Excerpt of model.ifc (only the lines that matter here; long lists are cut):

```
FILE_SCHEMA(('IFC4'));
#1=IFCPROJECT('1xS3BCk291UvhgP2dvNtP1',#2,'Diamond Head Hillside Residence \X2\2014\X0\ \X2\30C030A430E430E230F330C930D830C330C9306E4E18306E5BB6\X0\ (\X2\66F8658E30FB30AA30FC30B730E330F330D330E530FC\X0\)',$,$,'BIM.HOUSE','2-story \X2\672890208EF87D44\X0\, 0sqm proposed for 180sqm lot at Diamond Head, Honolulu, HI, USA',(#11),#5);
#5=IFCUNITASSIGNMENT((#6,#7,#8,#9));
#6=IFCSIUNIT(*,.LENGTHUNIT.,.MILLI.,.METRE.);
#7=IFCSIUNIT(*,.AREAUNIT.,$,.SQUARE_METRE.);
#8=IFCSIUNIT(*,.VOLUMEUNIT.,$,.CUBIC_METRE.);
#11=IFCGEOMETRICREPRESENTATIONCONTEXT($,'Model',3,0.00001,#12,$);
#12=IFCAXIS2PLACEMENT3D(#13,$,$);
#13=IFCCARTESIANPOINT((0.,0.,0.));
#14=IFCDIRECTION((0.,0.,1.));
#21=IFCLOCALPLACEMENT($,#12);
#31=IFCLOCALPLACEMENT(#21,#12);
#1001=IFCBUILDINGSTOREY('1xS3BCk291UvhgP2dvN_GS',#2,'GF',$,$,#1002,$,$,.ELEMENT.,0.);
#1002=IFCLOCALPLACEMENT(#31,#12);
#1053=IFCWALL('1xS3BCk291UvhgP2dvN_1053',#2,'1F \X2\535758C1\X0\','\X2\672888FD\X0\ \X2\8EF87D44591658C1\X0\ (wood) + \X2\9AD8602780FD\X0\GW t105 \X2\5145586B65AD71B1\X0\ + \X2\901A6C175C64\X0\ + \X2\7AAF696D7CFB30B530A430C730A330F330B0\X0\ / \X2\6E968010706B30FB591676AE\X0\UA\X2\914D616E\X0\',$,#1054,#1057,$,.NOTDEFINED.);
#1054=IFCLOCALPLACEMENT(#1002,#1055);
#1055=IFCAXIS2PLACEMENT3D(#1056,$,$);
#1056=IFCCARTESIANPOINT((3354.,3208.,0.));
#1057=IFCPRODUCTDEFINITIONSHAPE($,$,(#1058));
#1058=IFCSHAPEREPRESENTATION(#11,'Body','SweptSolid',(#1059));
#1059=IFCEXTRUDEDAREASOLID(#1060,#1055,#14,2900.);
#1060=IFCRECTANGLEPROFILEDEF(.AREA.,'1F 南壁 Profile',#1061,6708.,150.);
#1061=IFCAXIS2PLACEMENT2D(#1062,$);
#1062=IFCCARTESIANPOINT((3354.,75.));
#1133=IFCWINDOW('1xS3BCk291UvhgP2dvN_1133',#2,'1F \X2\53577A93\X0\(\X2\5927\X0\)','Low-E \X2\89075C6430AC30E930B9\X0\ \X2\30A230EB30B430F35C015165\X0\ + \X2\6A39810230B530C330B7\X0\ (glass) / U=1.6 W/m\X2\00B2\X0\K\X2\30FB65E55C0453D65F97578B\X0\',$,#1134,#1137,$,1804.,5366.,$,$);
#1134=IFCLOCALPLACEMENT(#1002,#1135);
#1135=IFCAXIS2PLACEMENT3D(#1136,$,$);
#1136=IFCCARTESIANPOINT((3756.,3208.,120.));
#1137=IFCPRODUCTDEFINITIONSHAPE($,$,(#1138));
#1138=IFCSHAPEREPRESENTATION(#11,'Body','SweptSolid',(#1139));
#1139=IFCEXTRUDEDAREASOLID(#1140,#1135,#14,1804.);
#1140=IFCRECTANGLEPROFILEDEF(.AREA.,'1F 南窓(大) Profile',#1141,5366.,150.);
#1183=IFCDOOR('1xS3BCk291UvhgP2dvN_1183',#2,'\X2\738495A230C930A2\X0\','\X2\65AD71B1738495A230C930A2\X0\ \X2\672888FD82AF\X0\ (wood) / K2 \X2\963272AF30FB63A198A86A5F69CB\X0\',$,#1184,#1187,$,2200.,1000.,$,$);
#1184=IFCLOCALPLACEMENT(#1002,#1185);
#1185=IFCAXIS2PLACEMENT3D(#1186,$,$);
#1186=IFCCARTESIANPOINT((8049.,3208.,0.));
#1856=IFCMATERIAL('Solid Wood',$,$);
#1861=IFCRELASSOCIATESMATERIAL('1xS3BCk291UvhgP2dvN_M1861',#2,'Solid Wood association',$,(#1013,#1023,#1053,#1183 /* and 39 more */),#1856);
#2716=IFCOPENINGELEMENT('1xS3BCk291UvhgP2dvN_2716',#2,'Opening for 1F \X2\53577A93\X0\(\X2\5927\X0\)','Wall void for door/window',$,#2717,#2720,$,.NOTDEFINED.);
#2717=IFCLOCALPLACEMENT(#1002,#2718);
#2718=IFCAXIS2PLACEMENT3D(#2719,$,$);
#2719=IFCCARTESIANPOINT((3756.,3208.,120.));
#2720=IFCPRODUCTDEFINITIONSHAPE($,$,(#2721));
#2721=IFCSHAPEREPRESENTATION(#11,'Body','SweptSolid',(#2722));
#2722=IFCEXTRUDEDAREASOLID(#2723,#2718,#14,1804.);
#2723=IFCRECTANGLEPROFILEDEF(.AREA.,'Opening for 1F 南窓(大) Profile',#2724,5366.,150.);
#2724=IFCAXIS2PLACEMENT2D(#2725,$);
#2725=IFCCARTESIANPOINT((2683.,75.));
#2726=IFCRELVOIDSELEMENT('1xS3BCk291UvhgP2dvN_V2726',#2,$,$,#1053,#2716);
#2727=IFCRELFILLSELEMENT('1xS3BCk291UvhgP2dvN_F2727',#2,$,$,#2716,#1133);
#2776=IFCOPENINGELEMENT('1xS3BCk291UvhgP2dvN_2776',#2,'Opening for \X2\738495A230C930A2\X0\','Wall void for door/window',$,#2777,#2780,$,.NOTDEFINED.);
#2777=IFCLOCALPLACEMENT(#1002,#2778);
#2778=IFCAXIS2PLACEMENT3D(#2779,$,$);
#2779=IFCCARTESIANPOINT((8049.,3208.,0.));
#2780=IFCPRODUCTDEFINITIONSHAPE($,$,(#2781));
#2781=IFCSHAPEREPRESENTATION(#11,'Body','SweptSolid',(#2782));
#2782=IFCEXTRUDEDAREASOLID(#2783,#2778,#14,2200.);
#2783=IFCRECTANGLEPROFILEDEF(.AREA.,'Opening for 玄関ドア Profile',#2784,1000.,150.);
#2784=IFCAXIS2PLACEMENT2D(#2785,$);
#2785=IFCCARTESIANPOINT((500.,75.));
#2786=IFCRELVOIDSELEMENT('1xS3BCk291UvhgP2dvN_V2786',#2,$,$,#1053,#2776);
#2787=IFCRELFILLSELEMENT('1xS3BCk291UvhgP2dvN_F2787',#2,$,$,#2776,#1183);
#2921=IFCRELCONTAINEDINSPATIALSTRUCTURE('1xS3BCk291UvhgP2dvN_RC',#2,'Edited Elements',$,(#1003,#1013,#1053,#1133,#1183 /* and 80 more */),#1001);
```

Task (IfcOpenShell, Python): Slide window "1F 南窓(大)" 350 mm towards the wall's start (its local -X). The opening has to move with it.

```python
import ifcopenshell
import ifcopenshell.api.geometry
import ifcopenshell.util.placement

model = ifcopenshell.open("model.ifc")

window = model.by_guid("1xS3BCk291UvhgP2dvN_1133")
opening = window.FillsVoids[0].RelatingOpeningElement
wall = opening.VoidsElements[0].RelatingBuildingElement

wall_matrix = ifcopenshell.util.placement.get_local_placement(wall.ObjectPlacement)
shift = wall_matrix[:3, 0] * -350.0
before = ifcopenshell.util.placement.get_local_placement(window.ObjectPlacement)[:3, 3].copy()

# The window is not placed relative to its opening, so move both.
for product in (opening, window):
    matrix = ifcopenshell.util.placement.get_local_placement(product.ObjectPlacement)
    matrix[:3, 3] += shift
    ifcopenshell.api.geometry.edit_object_placement(model, product=product, matrix=matrix, is_si=False)

after = ifcopenshell.util.placement.get_local_placement(window.ObjectPlacement)[:3, 3]
print("window moved by", (after - before).round(3) + 0.0)

model.write("model_v2.ifc")
```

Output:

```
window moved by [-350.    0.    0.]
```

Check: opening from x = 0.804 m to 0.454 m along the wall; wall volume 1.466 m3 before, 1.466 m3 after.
